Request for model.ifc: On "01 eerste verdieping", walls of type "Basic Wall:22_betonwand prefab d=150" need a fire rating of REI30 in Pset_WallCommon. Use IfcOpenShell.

First a look at what the model holds.

```python
import ifcopenshell
import ifcopenshell.util.element

model = ifcopenshell.open("model.ifc")
print(model.schema)
storey = next(s for s in model.by_type("IfcBuildingStorey") if s.Name == "01 eerste verdieping")
walls = [e for e in ifcopenshell.util.element.get_decomposition(storey) if e.is_a("IfcWall")]
seen = {}
for e in walls:
    element_type = ifcopenshell.util.element.get_type(e)
    key = (element_type.Name if element_type != e and element_type else None, ifcopenshell.util.element.get_pset(e, "Pset_WallCommon", "FireRating"))
    seen[key] = seen.get(key, 0) + 1
for (name, value), count in sorted(seen.items(), key=str):
    print(count, "x", name, "|", value)
```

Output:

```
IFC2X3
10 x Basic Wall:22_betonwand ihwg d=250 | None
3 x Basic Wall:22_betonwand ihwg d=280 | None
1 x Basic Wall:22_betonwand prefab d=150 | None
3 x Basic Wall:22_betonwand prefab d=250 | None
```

```python
import ifcopenshell
import ifcopenshell.api.pset
import ifcopenshell.util.element

model = ifcopenshell.open("model.ifc")

storey = next(s for s in model.by_type("IfcBuildingStorey") if s.Name == "01 eerste verdieping")
walls = [e for e in ifcopenshell.util.element.get_decomposition(storey) if e.is_a("IfcWall")]

count = 0
for e in walls:
    element_type = ifcopenshell.util.element.get_type(e)
    if element_type in (None, e) or element_type.Name != "Basic Wall:22_betonwand prefab d=150":
        continue
    # add_pset returns the element's existing set when there is one.
    pset = ifcopenshell.api.pset.add_pset(model, product=e, name="Pset_WallCommon")
    ifcopenshell.api.pset.edit_pset(model, pset=pset, properties={"FireRating": "REI30"})
    count += 1

print(count, "walls updated")

model.write("model_rev.ifc")
```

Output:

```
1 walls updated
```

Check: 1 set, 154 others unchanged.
